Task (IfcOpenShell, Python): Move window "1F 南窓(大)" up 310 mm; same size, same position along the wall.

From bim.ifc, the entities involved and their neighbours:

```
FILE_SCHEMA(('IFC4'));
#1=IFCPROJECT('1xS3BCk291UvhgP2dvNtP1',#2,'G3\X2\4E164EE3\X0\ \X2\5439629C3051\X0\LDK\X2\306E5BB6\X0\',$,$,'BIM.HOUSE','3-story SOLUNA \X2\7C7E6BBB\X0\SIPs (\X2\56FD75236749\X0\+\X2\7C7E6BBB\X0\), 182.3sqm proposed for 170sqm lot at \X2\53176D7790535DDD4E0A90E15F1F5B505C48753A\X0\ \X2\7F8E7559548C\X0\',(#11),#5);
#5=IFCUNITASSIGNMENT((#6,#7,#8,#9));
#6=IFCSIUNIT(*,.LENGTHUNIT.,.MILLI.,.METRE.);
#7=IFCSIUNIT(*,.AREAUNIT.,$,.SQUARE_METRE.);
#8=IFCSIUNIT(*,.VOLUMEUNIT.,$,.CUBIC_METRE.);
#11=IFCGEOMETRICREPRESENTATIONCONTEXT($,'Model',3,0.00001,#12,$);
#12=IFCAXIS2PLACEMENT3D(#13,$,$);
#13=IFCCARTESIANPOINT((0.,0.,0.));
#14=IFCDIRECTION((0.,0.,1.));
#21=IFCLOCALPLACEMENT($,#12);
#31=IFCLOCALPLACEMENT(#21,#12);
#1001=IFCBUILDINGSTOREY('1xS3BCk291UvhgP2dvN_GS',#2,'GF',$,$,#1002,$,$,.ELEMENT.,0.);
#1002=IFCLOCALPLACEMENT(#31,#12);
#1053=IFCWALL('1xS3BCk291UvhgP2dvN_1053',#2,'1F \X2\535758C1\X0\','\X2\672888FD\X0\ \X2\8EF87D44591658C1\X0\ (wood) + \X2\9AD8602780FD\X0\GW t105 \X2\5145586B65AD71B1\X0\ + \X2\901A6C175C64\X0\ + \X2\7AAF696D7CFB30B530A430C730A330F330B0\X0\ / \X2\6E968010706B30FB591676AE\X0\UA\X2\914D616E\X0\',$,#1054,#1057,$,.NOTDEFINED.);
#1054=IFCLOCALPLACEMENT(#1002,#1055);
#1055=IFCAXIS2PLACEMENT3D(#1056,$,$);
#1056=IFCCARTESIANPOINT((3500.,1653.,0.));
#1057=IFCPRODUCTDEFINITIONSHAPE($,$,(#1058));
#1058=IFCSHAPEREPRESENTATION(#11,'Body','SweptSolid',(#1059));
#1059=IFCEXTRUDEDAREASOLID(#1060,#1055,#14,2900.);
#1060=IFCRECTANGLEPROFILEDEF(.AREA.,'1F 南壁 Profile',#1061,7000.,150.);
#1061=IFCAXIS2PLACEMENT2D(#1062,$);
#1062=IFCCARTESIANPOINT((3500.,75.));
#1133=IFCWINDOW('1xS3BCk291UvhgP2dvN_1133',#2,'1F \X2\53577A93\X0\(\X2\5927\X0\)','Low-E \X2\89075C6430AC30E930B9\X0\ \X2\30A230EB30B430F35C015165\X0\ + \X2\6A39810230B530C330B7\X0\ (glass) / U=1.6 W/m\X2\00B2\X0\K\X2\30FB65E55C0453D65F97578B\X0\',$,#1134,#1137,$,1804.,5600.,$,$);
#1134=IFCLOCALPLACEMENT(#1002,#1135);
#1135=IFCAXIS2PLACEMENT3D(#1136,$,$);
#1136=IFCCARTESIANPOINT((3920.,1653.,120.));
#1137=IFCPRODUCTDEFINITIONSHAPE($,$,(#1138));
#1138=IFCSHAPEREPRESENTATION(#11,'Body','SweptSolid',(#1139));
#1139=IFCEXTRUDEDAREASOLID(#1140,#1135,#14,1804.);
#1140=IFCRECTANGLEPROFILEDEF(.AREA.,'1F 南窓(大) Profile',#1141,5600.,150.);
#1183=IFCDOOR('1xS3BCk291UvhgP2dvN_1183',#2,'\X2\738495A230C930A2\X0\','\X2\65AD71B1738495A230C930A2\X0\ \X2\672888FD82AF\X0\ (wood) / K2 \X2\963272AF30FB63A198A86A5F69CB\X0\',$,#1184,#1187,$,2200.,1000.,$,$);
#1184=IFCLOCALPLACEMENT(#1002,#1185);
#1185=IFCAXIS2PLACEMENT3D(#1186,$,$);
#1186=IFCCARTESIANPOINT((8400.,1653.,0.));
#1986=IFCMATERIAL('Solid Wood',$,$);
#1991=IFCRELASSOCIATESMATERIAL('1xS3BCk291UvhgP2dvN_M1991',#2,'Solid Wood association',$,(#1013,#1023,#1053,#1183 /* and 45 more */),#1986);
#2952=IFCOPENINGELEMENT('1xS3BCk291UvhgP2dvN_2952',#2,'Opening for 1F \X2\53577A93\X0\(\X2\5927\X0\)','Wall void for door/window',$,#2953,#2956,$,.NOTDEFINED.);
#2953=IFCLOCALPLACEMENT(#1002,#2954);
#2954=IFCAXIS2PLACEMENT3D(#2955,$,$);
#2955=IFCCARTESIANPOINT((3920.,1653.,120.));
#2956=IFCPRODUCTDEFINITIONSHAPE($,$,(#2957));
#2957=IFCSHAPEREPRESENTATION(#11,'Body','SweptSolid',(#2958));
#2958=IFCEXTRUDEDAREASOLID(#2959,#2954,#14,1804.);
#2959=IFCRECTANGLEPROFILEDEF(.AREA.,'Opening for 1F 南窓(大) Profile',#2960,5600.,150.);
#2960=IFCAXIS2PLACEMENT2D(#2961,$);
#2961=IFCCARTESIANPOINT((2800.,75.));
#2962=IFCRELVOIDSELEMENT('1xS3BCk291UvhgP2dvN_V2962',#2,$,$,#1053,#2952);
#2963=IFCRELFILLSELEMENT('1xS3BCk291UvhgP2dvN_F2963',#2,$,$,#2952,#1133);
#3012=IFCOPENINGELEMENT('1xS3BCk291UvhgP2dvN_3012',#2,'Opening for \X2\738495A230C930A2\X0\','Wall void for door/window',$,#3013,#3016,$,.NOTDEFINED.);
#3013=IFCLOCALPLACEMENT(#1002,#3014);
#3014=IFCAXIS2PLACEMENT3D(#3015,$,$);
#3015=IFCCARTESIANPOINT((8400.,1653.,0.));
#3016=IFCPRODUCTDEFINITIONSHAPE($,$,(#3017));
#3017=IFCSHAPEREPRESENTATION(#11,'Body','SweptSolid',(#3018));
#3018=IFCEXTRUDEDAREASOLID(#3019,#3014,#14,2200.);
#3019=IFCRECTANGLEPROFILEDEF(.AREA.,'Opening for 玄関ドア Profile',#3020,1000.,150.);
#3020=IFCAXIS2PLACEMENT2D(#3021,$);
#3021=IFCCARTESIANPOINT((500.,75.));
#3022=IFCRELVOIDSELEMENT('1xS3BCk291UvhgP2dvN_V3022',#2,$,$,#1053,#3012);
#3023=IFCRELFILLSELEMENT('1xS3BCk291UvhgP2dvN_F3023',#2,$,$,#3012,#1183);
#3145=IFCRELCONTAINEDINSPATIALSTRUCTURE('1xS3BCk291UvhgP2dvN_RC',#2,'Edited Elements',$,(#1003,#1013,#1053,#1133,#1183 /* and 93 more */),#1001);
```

```python
import numpy as np
import ifcopenshell
import ifcopenshell.api.geometry
import ifcopenshell.util.placement
import ifcopenshell.util.unit

model = ifcopenshell.open("bim.ifc")
unit_scale = ifcopenshell.util.unit.calculate_unit_scale(model)

window = model.by_guid("1xS3BCk291UvhgP2dvN_1133")
opening = window.FillsVoids[0].RelatingOpeningElement
dz = 0.31 / unit_scale

shift = np.array([0.0, 0.0, dz])
# The window is not placed relative to its opening, so move both.
for product in (opening, window):
    matrix = ifcopenshell.util.placement.get_local_placement(product.ObjectPlacement)
    matrix[:3, 3] += shift
    ifcopenshell.api.geometry.edit_object_placement(model, product=product, matrix=matrix, is_si=False)

print(f"moved by {dz * unit_scale:+.3f} m")

model.write("bim-out.ifc")
```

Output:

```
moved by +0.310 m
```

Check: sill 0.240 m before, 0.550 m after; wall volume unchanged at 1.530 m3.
